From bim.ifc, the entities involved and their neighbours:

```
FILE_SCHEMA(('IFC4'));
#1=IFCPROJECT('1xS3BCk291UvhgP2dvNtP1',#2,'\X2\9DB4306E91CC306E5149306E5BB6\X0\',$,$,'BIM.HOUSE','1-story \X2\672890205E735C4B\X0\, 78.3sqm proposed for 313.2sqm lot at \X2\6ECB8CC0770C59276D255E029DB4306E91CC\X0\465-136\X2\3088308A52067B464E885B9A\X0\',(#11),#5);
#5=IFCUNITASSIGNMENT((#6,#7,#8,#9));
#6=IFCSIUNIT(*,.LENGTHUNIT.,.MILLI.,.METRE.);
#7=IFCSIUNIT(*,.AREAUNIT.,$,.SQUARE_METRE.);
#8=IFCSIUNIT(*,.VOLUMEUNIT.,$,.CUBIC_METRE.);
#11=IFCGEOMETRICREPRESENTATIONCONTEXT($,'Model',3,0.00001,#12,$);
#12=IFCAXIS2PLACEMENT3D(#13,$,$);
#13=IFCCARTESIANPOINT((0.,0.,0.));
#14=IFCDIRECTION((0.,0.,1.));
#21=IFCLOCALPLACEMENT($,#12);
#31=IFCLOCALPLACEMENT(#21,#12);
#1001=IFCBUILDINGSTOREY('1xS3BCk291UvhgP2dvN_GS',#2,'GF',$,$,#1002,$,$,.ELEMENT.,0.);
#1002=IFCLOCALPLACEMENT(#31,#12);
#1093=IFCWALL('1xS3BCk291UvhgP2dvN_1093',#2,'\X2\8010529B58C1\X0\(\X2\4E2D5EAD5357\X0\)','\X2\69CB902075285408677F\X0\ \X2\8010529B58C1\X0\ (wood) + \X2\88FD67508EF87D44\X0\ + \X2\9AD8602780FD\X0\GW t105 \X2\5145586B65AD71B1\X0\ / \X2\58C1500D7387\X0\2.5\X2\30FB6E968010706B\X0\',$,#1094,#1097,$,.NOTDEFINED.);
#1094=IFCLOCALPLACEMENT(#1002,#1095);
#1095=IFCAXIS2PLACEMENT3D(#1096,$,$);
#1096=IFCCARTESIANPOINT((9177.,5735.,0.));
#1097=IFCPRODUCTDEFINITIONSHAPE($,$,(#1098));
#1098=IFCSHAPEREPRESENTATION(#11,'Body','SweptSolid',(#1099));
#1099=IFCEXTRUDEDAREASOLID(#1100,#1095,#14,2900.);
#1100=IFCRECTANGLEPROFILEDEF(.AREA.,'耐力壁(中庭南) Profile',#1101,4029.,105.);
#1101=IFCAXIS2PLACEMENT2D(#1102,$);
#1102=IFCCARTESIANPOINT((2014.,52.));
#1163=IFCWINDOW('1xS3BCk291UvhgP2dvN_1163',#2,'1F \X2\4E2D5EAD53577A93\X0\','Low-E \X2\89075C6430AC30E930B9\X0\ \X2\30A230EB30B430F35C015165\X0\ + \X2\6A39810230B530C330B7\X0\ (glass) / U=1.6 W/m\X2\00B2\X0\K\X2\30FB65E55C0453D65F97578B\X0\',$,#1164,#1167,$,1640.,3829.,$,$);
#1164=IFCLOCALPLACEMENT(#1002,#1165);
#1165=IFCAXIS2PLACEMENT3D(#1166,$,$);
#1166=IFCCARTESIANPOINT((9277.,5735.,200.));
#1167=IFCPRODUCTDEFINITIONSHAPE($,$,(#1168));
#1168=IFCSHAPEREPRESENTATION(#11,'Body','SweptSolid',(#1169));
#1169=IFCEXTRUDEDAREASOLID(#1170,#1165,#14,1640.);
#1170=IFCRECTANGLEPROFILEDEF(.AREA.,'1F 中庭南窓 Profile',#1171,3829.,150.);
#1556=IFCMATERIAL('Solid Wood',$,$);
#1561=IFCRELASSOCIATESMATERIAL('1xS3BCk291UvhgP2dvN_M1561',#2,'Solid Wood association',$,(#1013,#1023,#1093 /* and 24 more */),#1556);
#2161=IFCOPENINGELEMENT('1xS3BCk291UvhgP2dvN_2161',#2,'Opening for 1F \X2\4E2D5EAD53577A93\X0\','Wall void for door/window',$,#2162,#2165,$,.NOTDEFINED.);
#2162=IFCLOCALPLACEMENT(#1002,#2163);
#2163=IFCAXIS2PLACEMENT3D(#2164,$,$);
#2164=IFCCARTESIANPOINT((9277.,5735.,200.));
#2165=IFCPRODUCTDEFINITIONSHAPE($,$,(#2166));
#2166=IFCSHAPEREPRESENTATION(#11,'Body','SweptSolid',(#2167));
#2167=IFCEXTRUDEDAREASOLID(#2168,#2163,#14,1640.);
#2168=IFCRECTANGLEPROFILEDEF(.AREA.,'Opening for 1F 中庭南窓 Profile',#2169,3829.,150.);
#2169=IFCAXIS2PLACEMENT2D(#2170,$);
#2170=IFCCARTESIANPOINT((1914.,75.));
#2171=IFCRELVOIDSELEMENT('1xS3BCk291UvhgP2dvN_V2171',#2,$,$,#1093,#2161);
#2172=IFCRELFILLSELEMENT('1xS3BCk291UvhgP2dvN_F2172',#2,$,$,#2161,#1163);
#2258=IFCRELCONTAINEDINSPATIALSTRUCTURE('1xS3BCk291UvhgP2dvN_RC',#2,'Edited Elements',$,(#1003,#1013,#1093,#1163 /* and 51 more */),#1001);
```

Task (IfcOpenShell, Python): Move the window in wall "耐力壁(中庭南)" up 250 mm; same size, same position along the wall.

```python
import numpy as np
import ifcopenshell
import ifcopenshell.api.geometry
import ifcopenshell.util.placement
import ifcopenshell.util.unit

model = ifcopenshell.open("bim.ifc")
unit_scale = ifcopenshell.util.unit.calculate_unit_scale(model)

window = model.by_guid("1xS3BCk291UvhgP2dvN_1163")
opening = window.FillsVoids[0].RelatingOpeningElement
dz = 0.25 / unit_scale

shift = np.array([0.0, 0.0, dz])
# The window is not placed relative to its opening, so move both.
for product in (opening, window):
    matrix = ifcopenshell.util.placement.get_local_placement(product.ObjectPlacement)
    matrix[:3, 3] += shift
    ifcopenshell.api.geometry.edit_object_placement(model, product=product, matrix=matrix, is_si=False)

print(f"moved by {dz * unit_scale:+.3f} m")

model.write("bim_rev.ifc")
```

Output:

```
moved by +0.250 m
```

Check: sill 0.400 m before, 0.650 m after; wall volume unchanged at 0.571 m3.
